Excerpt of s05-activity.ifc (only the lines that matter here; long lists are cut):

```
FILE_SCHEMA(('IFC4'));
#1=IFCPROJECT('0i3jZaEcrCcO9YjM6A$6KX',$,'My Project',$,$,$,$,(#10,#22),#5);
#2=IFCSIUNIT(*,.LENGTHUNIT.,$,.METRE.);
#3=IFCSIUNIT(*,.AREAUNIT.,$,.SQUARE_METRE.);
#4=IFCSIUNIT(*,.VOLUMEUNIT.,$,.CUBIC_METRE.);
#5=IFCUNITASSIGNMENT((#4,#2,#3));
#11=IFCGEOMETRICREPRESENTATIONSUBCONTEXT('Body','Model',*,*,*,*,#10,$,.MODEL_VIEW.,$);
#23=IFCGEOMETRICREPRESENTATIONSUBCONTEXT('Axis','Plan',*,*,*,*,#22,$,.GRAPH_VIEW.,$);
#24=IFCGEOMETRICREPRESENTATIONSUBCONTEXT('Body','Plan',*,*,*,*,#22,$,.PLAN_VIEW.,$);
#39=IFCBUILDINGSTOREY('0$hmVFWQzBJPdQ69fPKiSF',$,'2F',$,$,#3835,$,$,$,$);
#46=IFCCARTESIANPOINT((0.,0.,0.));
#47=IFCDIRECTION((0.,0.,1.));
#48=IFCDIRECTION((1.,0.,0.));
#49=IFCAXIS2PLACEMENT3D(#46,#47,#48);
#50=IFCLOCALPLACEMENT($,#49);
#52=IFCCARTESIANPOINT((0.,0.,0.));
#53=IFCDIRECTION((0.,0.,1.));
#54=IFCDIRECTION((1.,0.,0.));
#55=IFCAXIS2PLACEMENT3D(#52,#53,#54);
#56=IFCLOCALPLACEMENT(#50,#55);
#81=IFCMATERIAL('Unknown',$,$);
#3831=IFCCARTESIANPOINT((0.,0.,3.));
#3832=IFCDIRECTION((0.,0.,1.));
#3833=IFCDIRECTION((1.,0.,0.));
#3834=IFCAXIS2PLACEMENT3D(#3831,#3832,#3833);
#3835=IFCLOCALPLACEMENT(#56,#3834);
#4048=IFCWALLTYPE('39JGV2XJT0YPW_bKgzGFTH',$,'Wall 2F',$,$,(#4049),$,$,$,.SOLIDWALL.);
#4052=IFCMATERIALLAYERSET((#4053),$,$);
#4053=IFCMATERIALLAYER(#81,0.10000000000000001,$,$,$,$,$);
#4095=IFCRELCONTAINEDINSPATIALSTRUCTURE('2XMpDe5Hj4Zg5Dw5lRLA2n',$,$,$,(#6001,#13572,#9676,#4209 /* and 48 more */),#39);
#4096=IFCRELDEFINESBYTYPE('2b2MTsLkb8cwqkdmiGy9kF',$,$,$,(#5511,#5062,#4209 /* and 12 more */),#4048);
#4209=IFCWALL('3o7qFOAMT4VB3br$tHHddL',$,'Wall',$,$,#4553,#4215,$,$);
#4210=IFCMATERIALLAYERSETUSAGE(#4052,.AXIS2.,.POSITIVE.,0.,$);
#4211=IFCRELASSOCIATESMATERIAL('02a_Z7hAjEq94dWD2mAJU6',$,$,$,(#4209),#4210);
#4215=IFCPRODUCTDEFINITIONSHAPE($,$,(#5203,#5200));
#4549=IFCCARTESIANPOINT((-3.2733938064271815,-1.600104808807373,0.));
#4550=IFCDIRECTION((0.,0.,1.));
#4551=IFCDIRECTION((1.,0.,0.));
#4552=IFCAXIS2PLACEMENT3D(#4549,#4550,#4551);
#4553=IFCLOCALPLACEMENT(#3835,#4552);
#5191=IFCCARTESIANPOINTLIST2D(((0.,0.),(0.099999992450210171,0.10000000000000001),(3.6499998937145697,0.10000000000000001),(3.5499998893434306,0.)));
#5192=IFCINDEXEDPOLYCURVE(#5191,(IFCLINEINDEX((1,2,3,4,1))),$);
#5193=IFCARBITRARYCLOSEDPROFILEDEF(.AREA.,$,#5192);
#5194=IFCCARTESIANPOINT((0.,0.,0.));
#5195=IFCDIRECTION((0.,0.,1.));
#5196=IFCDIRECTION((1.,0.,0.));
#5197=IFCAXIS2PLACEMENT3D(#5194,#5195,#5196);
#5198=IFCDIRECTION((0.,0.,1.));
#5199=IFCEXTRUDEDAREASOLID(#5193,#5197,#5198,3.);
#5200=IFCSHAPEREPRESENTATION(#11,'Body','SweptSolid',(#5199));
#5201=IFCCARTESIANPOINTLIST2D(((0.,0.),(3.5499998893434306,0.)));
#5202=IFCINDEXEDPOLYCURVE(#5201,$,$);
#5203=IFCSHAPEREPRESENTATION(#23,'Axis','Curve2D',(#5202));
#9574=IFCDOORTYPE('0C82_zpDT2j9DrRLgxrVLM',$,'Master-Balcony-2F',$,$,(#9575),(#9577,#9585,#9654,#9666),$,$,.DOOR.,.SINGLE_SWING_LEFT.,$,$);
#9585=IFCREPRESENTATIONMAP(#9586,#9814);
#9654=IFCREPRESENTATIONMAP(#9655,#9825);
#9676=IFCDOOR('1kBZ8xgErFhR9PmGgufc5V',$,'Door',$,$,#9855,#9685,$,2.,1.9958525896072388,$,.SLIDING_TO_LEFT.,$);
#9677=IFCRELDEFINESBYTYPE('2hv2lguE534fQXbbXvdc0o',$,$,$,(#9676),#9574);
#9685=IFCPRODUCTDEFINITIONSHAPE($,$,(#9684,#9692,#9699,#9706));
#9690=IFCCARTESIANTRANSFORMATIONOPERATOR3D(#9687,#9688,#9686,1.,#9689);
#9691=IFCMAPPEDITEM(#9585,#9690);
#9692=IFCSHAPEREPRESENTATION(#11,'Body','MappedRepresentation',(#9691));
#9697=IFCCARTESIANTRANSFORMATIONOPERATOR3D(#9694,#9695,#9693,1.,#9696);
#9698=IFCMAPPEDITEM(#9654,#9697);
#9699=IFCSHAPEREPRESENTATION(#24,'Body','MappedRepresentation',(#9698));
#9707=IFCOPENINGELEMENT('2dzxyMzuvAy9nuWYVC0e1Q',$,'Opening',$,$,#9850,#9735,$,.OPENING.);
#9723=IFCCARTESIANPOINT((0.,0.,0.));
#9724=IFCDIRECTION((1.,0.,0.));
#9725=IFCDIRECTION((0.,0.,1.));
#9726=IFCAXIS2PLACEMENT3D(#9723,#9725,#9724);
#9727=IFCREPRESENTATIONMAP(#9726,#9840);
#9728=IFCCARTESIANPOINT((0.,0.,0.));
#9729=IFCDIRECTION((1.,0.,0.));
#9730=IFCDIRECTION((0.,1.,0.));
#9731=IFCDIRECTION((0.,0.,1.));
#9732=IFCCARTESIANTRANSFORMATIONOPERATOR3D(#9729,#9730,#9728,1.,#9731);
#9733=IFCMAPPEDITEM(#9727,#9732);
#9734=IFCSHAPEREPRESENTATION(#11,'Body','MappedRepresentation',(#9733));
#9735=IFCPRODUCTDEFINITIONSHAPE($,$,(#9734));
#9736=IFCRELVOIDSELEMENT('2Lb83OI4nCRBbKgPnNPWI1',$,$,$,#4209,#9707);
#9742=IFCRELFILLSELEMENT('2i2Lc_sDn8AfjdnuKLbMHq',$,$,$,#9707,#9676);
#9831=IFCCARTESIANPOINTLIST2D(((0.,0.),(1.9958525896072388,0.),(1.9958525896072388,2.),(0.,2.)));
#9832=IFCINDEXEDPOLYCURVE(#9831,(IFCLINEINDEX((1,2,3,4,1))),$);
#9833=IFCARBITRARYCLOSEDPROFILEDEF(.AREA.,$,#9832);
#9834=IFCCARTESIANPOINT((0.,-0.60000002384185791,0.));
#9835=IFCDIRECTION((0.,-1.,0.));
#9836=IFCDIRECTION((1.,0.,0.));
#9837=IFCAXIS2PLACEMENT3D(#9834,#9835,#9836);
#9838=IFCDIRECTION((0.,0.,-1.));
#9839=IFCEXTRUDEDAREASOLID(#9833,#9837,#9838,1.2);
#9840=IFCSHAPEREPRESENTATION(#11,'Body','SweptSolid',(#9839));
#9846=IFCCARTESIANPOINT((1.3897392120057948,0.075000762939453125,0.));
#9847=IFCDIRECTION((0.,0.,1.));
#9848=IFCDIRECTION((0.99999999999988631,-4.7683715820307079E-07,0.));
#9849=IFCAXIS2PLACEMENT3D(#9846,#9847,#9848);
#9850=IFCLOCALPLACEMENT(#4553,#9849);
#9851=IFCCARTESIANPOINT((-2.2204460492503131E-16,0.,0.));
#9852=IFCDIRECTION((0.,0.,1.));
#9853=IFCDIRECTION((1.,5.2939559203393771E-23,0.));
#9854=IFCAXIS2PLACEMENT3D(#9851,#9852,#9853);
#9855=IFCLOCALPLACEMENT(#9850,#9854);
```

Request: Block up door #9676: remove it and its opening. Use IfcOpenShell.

```python
import ifcopenshell
import ifcopenshell.api.feature
import ifcopenshell.api.root
import ifcopenshell.geom
import ifcopenshell.util.shape

model = ifcopenshell.open("s05-activity.ifc")
settings = ifcopenshell.geom.settings()


def volume(element):
    """Net volume in cubic metres, openings subtracted."""
    shape = ifcopenshell.geom.create_shape(settings, element)
    return ifcopenshell.util.shape.get_volume(shape.geometry)


door = model.by_guid("1kBZ8xgErFhR9PmGgufc5V")
opening = door.FillsVoids[0].RelatingOpeningElement
wall = opening.VoidsElements[0].RelatingBuildingElement
before = volume(wall)

ifcopenshell.api.root.remove_product(model, product=door)
ifcopenshell.api.feature.remove_feature(model, feature=opening)

after = volume(wall)

print(f"wall volume {before:.3f} -> {after:.3f} m3")

model.write("s05-activity_updated.ifc")
```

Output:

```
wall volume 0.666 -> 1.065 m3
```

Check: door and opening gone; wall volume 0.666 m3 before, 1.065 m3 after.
